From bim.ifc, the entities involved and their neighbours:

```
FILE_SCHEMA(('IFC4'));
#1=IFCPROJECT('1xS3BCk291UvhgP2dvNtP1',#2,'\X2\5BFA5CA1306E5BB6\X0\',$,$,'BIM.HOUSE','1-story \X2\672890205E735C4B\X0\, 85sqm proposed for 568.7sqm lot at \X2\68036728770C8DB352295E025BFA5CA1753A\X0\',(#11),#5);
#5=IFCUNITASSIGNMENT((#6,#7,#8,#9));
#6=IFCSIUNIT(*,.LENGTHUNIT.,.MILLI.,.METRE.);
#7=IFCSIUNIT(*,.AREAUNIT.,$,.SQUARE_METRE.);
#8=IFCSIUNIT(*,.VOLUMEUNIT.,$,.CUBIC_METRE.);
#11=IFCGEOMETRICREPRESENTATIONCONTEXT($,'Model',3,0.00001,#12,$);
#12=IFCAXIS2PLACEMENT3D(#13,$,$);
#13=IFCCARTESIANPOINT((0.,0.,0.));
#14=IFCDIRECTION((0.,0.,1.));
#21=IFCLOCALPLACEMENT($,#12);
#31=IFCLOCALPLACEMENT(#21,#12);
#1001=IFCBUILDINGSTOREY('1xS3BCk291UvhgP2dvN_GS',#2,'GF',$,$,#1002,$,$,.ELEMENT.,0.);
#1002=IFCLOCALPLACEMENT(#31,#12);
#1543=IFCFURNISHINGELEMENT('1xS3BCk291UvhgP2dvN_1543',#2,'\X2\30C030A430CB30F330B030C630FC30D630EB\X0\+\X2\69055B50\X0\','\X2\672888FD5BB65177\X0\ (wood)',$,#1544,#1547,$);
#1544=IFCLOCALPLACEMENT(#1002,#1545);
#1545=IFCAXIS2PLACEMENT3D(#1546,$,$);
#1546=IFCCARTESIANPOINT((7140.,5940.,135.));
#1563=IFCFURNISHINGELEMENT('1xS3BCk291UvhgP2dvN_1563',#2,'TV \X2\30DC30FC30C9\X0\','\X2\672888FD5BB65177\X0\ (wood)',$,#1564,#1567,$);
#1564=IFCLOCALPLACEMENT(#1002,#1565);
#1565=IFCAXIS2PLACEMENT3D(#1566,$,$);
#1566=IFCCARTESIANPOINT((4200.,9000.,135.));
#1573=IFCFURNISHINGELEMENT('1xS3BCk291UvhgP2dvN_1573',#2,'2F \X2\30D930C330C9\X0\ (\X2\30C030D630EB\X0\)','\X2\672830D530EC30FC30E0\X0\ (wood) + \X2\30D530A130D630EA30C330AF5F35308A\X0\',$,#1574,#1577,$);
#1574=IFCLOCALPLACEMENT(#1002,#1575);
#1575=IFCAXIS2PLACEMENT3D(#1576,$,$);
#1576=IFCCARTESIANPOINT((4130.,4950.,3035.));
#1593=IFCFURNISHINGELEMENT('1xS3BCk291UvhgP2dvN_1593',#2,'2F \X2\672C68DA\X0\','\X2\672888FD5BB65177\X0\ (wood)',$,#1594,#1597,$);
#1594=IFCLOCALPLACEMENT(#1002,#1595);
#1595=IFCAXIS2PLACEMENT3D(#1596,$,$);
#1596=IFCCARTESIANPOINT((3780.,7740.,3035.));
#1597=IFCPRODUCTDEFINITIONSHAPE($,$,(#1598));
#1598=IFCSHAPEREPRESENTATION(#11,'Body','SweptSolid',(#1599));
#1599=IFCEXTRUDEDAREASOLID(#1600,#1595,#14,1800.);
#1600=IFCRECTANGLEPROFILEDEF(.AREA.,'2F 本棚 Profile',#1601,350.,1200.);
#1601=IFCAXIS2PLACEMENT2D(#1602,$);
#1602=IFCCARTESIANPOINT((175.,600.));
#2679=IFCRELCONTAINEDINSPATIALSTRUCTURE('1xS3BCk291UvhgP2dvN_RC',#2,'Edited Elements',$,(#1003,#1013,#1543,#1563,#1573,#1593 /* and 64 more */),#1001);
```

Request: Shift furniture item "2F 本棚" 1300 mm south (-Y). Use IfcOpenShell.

```python
import ifcopenshell
import ifcopenshell.api.geometry
import ifcopenshell.util.placement

model = ifcopenshell.open("bim.ifc")

item = model.by_id(1593)
matrix = ifcopenshell.util.placement.get_local_placement(item.ObjectPlacement)
matrix[1, 3] -= 1300.0
ifcopenshell.api.geometry.edit_object_placement(model, product=item, matrix=matrix, is_si=False)

print(ifcopenshell.util.placement.get_local_placement(item.ObjectPlacement).round(3) + 0.0)

model.write("bim_updated.ifc")
```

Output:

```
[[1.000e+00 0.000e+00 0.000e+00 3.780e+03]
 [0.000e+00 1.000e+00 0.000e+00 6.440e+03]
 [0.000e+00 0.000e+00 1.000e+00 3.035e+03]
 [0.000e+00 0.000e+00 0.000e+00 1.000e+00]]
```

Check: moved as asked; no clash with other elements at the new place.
